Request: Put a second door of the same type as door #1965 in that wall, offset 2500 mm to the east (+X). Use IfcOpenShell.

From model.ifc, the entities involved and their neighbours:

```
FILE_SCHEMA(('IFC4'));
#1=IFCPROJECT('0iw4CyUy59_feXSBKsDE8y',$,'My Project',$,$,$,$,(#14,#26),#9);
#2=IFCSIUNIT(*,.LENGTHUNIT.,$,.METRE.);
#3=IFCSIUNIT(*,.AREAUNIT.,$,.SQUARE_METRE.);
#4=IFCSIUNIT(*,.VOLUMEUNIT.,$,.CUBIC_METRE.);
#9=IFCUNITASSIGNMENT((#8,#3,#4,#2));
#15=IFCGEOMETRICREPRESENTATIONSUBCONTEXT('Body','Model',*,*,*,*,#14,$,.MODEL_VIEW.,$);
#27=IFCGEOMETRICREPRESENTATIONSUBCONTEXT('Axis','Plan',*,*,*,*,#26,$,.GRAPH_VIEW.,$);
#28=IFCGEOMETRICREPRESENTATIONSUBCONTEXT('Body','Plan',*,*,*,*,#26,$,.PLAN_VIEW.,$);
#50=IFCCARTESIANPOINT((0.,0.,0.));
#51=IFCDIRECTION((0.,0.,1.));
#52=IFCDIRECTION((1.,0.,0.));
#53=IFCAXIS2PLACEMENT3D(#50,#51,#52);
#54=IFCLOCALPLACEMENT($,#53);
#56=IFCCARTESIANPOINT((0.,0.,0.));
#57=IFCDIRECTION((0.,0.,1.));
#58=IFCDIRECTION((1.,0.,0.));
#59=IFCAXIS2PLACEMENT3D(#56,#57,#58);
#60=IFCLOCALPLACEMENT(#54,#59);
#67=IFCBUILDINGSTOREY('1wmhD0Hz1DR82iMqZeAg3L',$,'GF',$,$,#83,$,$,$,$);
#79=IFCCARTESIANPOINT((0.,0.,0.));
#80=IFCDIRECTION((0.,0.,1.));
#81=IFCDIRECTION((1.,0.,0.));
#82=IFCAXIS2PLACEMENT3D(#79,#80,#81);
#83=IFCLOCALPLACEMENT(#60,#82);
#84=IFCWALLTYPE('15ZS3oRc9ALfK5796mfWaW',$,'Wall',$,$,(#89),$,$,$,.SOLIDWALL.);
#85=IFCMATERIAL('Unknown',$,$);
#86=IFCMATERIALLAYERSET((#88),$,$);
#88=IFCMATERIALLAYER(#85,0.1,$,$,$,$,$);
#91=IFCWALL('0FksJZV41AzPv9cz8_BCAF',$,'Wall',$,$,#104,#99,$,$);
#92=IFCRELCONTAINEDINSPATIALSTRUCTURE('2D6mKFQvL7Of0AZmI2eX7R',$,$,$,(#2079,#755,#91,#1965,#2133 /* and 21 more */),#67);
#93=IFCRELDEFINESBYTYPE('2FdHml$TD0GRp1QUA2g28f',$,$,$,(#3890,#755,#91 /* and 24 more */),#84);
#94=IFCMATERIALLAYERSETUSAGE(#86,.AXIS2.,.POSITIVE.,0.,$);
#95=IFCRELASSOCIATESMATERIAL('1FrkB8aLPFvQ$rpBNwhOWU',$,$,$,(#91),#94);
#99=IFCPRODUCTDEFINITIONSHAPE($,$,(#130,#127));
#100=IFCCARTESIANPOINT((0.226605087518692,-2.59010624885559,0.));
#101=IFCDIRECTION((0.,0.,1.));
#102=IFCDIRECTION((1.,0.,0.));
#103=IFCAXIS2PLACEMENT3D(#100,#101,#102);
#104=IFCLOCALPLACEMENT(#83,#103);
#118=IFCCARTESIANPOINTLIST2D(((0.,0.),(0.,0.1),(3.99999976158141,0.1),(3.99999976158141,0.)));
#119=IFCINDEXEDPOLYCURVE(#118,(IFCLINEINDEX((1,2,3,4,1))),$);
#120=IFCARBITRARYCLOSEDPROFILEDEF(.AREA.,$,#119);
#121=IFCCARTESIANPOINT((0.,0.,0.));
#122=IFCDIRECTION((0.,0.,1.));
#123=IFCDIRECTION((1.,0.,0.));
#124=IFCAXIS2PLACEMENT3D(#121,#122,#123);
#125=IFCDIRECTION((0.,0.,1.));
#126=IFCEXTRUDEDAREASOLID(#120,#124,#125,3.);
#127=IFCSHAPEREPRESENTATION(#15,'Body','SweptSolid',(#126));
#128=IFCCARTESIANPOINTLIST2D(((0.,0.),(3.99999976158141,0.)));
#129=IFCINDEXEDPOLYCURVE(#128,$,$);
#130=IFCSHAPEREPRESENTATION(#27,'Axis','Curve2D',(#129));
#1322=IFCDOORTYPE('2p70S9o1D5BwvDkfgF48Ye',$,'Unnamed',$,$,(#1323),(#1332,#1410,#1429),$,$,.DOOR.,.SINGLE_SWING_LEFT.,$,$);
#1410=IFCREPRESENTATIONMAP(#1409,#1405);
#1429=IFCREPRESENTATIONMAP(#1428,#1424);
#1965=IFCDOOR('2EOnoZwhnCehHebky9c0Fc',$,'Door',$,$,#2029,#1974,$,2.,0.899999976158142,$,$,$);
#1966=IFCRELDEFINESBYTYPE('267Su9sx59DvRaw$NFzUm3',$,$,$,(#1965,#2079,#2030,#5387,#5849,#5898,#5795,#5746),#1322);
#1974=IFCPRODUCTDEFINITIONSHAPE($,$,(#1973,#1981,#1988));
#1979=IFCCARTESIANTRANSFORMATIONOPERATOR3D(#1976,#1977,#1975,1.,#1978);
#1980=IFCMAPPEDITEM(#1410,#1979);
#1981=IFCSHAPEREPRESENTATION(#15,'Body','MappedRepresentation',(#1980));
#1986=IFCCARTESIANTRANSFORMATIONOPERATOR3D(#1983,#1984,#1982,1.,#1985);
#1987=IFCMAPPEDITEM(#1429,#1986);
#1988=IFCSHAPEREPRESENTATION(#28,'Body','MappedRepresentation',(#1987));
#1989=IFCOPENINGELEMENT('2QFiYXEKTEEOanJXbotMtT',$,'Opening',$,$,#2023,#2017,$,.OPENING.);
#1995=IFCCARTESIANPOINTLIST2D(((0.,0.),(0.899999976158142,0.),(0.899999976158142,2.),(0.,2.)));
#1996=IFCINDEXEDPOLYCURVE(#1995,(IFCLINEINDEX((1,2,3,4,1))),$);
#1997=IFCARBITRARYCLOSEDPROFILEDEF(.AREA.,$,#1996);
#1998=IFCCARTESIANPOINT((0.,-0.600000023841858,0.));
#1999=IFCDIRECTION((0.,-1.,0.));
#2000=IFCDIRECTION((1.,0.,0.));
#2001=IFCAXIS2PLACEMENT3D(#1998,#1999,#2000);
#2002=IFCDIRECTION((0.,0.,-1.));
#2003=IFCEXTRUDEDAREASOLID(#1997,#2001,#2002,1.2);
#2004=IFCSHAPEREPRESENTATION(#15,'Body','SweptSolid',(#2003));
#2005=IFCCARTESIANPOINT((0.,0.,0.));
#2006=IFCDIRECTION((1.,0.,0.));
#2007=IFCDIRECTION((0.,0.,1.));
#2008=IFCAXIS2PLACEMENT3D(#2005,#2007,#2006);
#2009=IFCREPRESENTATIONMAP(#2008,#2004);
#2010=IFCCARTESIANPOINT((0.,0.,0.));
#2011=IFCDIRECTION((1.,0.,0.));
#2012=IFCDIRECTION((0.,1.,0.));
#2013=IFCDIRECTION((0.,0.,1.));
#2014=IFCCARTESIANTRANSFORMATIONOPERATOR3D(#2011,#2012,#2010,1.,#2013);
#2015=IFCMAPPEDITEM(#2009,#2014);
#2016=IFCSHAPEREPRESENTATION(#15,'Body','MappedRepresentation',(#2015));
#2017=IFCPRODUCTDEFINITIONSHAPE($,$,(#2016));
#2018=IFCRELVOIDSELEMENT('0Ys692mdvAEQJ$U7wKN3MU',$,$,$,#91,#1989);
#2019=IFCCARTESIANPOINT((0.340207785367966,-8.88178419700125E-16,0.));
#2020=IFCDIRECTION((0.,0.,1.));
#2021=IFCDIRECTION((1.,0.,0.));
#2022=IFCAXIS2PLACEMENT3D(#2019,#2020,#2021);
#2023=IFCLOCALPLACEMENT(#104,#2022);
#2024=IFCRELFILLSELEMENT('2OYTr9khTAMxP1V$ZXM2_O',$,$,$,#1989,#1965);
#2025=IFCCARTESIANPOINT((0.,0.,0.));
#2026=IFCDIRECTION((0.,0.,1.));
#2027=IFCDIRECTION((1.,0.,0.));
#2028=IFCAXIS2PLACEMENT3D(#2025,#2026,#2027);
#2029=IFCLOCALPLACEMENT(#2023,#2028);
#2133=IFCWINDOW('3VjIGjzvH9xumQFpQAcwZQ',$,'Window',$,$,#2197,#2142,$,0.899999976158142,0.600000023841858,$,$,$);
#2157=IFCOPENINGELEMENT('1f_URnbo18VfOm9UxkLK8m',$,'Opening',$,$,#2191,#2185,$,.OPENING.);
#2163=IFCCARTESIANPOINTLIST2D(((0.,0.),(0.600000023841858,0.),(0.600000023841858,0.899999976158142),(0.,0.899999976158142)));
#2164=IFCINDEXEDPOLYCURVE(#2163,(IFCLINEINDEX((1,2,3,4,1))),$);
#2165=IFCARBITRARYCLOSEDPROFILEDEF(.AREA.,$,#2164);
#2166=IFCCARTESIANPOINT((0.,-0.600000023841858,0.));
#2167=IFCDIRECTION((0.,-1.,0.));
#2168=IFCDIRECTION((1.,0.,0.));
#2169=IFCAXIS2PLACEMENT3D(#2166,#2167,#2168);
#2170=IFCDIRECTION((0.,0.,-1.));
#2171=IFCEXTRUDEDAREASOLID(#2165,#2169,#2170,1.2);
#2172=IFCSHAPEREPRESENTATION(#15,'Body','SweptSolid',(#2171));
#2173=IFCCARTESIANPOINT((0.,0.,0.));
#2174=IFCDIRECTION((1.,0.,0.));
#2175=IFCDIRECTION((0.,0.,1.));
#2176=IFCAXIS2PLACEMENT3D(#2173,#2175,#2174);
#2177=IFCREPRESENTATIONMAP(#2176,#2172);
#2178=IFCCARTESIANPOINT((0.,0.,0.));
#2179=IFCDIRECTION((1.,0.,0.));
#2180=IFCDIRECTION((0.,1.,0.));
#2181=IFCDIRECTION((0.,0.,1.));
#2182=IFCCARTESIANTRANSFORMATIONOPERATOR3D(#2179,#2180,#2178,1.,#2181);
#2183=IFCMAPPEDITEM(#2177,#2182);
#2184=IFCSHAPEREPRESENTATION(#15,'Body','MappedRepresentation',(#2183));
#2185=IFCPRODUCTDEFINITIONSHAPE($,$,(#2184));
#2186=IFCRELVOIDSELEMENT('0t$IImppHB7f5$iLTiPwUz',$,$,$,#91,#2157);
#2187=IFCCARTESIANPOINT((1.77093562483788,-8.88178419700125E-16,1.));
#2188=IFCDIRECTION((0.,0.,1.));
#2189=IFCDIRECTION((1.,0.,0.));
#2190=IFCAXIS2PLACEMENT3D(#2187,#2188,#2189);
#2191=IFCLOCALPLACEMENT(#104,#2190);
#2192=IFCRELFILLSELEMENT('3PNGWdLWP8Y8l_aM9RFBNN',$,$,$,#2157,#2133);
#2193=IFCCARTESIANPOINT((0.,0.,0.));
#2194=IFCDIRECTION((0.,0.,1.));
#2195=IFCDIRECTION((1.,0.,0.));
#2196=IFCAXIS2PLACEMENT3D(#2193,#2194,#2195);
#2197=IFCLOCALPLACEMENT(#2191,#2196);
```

```python
import ifcopenshell
import ifcopenshell.api.feature
import ifcopenshell.api.geometry
import ifcopenshell.api.root
import ifcopenshell.geom
import ifcopenshell.util.element
import ifcopenshell.util.placement
import ifcopenshell.util.shape

model = ifcopenshell.open("model.ifc")
settings = ifcopenshell.geom.settings()


def volume(element):
    """Net volume in cubic metres, openings subtracted."""
    shape = ifcopenshell.geom.create_shape(settings, element)
    return ifcopenshell.util.shape.get_volume(shape.geometry)


door = model.by_guid("2EOnoZwhnCehHebky9c0Fc")
opening = door.FillsVoids[0].RelatingOpeningElement
wall = opening.VoidsElements[0].RelatingBuildingElement
before = volume(wall)
shift = ifcopenshell.util.placement.get_local_placement(wall.ObjectPlacement)[:3, 0] * 2.5

# copy_class copies the void relationship, type, container and properties, but no geometry.
new_opening = ifcopenshell.api.root.copy_class(model, product=opening)
new_opening.Representation = ifcopenshell.util.element.copy_deep(
    model, opening.Representation, exclude=["IfcGeometricRepresentationContext", "IfcRepresentationMap"]
)
new_door = ifcopenshell.api.root.copy_class(model, product=door)
new_door.Representation = ifcopenshell.util.element.copy_deep(
    model, door.Representation, exclude=["IfcGeometricRepresentationContext", "IfcRepresentationMap"]
)
ifcopenshell.api.feature.add_filling(model, opening=new_opening, element=new_door)

for old, new in ((opening, new_opening), (door, new_door)):
    matrix = ifcopenshell.util.placement.get_local_placement(old.ObjectPlacement)
    matrix[:3, 3] += shift
    ifcopenshell.api.geometry.edit_object_placement(model, product=new, matrix=matrix, is_si=False)

after = volume(wall)

print(f"wall volume {before:.3f} -> {after:.3f} m3")

model.write("model-out.ifc")
```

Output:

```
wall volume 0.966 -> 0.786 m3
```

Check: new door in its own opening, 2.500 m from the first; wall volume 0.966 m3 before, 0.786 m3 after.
